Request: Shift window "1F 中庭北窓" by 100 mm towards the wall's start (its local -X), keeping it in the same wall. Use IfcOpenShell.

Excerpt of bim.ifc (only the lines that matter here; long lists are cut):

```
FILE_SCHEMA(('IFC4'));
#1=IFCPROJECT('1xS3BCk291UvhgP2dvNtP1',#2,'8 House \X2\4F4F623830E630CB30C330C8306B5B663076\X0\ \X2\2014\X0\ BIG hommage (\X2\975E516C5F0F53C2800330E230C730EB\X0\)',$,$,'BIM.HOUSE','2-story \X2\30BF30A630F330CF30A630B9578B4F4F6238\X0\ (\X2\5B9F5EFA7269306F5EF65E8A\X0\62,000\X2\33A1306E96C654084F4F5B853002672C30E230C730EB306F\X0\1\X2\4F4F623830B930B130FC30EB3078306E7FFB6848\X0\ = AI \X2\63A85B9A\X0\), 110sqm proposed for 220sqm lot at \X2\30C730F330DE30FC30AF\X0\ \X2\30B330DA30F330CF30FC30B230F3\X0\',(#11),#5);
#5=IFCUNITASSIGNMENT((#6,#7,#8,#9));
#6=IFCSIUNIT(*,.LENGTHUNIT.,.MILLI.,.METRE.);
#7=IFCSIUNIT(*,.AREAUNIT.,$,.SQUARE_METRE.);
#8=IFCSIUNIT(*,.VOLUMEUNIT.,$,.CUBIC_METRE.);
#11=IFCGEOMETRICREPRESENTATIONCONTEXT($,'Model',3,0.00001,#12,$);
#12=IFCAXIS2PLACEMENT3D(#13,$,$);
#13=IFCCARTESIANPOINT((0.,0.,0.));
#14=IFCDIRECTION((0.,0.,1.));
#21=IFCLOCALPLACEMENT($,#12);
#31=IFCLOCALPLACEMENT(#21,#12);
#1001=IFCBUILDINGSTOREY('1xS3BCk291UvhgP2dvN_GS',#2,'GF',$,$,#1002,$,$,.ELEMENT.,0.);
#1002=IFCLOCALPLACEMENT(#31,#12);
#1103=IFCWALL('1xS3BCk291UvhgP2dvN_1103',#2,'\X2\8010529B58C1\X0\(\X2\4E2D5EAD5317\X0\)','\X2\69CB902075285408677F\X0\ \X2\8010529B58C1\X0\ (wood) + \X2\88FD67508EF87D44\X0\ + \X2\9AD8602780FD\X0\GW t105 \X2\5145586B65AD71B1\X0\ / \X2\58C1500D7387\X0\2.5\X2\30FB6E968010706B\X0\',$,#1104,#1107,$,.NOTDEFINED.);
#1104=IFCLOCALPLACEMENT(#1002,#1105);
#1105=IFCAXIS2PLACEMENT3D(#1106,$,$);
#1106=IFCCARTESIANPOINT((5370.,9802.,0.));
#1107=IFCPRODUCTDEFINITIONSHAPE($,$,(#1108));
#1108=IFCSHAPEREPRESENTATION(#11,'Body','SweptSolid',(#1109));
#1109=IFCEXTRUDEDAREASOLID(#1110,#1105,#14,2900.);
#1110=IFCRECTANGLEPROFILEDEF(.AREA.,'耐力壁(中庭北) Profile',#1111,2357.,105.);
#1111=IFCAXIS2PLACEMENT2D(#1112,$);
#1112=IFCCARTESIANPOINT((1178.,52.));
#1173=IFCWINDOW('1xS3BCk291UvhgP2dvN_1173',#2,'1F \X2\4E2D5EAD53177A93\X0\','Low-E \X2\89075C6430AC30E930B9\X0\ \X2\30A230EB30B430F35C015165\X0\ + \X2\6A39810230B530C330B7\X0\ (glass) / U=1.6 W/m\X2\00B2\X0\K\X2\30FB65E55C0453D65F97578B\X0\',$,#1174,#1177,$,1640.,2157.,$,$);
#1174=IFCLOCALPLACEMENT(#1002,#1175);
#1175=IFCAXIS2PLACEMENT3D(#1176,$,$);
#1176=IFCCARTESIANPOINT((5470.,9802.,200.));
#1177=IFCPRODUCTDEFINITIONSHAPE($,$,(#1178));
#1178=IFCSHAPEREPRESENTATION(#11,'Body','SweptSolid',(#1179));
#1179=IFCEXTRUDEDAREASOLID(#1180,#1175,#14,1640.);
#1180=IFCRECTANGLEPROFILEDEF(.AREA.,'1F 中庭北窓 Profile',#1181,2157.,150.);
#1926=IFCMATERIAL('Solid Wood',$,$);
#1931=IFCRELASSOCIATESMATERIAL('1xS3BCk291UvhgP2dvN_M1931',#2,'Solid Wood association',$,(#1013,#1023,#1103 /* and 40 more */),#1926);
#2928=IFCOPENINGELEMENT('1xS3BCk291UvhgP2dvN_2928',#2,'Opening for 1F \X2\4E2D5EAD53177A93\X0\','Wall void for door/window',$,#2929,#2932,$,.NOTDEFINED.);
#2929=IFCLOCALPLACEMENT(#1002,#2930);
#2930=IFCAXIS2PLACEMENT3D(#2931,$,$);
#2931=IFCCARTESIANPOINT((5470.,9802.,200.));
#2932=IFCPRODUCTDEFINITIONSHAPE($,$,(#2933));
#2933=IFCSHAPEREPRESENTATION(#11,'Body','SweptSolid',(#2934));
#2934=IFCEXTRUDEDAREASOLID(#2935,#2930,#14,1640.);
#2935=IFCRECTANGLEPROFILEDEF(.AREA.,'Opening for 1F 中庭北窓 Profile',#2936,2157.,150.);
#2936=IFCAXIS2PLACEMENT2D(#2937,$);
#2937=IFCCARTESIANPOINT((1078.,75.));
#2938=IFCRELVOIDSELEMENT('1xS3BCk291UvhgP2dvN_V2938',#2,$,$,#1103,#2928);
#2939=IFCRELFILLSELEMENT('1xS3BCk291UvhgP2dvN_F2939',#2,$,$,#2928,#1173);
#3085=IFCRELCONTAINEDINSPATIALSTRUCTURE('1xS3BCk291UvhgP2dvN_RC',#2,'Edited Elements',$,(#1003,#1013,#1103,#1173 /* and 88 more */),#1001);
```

```python
import ifcopenshell
import ifcopenshell.api.geometry
import ifcopenshell.util.placement
import ifcopenshell.util.unit

model = ifcopenshell.open("bim.ifc")
unit_scale = ifcopenshell.util.unit.calculate_unit_scale(model)

window = model.by_guid("1xS3BCk291UvhgP2dvN_1173")
opening = window.FillsVoids[0].RelatingOpeningElement
wall = opening.VoidsElements[0].RelatingBuildingElement

wall_matrix = ifcopenshell.util.placement.get_local_placement(wall.ObjectPlacement)
shift = wall_matrix[:3, 0] * -0.1 / unit_scale
before = ifcopenshell.util.placement.get_local_placement(window.ObjectPlacement)[:3, 3].copy()

# The window is not placed relative to its opening, so move both.
for product in (opening, window):
    matrix = ifcopenshell.util.placement.get_local_placement(product.ObjectPlacement)
    matrix[:3, 3] += shift
    ifcopenshell.api.geometry.edit_object_placement(model, product=product, matrix=matrix, is_si=False)

after = ifcopenshell.util.placement.get_local_placement(window.ObjectPlacement)[:3, 3]
print("window moved by", (after - before).round(3) + 0.0)

model.write("bim_edited.ifc")
```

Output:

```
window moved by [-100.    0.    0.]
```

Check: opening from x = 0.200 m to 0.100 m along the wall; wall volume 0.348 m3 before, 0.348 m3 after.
